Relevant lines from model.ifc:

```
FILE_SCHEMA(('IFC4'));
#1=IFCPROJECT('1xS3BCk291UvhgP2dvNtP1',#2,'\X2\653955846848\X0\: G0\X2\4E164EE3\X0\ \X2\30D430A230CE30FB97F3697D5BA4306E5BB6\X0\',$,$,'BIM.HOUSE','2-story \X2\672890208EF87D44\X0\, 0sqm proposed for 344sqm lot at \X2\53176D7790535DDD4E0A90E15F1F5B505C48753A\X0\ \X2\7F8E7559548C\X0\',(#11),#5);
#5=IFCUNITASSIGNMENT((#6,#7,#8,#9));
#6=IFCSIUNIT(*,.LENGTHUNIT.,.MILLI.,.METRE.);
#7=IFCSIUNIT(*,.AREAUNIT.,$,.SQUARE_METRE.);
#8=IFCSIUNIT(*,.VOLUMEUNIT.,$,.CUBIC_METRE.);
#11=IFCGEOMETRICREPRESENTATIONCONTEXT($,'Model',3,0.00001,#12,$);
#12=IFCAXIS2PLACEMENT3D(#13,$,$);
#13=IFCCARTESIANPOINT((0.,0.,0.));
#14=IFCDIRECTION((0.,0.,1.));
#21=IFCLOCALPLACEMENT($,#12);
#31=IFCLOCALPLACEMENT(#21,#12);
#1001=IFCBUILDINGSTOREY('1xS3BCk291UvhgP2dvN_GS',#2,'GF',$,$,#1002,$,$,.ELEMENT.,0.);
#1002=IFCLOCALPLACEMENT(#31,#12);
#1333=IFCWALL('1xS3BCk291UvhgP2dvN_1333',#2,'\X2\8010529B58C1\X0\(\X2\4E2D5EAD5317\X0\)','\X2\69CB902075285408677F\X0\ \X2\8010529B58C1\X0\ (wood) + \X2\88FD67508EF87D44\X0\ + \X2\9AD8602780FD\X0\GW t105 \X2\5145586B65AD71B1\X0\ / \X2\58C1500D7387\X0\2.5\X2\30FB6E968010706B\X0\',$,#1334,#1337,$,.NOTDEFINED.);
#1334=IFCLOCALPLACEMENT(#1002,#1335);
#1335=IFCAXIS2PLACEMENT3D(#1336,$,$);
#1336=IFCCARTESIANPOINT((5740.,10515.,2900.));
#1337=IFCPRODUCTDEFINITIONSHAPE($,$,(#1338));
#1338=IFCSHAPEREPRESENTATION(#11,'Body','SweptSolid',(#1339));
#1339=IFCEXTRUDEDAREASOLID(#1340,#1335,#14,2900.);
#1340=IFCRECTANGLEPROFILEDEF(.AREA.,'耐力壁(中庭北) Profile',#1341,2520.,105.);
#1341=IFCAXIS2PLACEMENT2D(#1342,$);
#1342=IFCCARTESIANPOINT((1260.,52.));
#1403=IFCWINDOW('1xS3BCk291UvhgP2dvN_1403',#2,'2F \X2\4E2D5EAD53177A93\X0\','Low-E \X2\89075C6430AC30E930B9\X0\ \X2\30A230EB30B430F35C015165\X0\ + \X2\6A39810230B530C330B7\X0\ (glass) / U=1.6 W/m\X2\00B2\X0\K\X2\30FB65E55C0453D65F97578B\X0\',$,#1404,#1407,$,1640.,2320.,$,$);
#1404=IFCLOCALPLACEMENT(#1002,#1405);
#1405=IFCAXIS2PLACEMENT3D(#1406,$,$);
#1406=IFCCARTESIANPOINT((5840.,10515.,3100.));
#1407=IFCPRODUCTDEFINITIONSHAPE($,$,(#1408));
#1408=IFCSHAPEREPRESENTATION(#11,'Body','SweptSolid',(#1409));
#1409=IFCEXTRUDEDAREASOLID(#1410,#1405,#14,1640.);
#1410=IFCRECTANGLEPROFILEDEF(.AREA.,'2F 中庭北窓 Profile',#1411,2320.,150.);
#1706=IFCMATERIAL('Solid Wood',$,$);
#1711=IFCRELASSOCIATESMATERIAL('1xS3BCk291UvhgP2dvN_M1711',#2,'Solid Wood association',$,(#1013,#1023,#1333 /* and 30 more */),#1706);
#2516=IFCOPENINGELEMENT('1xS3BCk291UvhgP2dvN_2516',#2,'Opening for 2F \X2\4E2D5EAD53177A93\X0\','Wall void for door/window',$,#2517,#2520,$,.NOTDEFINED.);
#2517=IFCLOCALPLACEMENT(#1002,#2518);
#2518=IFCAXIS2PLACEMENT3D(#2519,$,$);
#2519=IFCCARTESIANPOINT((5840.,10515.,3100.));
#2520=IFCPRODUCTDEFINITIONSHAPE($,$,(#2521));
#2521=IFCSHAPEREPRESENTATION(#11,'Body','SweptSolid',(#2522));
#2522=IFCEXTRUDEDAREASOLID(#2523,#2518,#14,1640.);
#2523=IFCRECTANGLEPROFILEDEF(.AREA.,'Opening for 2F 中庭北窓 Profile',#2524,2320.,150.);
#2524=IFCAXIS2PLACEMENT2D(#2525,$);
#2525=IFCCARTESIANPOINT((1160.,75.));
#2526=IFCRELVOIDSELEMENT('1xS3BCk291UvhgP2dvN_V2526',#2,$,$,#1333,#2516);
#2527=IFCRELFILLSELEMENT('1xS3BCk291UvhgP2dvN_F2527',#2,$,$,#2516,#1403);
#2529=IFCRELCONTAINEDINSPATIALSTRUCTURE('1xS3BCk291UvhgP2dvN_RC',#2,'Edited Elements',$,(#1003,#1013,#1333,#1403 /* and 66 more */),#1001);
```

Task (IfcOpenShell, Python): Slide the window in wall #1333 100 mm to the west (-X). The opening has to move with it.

```python
import ifcopenshell
import ifcopenshell.api.geometry
import ifcopenshell.util.placement
import ifcopenshell.util.unit

model = ifcopenshell.open("model.ifc")
unit_scale = ifcopenshell.util.unit.calculate_unit_scale(model)

window = model.by_id(1403)
opening = window.FillsVoids[0].RelatingOpeningElement
wall = opening.VoidsElements[0].RelatingBuildingElement

wall_matrix = ifcopenshell.util.placement.get_local_placement(wall.ObjectPlacement)
shift = wall_matrix[:3, 0] * -0.1 / unit_scale
before = ifcopenshell.util.placement.get_local_placement(window.ObjectPlacement)[:3, 3].copy()

# The window is not placed relative to its opening, so move both.
for product in (opening, window):
    matrix = ifcopenshell.util.placement.get_local_placement(product.ObjectPlacement)
    matrix[:3, 3] += shift
    ifcopenshell.api.geometry.edit_object_placement(model, product=product, matrix=matrix, is_si=False)

after = ifcopenshell.util.placement.get_local_placement(window.ObjectPlacement)[:3, 3]
print("window moved by", (after - before).round(3) + 0.0)

model.write("model-out.ifc")
```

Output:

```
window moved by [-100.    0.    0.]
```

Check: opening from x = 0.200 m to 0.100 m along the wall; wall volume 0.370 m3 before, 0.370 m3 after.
